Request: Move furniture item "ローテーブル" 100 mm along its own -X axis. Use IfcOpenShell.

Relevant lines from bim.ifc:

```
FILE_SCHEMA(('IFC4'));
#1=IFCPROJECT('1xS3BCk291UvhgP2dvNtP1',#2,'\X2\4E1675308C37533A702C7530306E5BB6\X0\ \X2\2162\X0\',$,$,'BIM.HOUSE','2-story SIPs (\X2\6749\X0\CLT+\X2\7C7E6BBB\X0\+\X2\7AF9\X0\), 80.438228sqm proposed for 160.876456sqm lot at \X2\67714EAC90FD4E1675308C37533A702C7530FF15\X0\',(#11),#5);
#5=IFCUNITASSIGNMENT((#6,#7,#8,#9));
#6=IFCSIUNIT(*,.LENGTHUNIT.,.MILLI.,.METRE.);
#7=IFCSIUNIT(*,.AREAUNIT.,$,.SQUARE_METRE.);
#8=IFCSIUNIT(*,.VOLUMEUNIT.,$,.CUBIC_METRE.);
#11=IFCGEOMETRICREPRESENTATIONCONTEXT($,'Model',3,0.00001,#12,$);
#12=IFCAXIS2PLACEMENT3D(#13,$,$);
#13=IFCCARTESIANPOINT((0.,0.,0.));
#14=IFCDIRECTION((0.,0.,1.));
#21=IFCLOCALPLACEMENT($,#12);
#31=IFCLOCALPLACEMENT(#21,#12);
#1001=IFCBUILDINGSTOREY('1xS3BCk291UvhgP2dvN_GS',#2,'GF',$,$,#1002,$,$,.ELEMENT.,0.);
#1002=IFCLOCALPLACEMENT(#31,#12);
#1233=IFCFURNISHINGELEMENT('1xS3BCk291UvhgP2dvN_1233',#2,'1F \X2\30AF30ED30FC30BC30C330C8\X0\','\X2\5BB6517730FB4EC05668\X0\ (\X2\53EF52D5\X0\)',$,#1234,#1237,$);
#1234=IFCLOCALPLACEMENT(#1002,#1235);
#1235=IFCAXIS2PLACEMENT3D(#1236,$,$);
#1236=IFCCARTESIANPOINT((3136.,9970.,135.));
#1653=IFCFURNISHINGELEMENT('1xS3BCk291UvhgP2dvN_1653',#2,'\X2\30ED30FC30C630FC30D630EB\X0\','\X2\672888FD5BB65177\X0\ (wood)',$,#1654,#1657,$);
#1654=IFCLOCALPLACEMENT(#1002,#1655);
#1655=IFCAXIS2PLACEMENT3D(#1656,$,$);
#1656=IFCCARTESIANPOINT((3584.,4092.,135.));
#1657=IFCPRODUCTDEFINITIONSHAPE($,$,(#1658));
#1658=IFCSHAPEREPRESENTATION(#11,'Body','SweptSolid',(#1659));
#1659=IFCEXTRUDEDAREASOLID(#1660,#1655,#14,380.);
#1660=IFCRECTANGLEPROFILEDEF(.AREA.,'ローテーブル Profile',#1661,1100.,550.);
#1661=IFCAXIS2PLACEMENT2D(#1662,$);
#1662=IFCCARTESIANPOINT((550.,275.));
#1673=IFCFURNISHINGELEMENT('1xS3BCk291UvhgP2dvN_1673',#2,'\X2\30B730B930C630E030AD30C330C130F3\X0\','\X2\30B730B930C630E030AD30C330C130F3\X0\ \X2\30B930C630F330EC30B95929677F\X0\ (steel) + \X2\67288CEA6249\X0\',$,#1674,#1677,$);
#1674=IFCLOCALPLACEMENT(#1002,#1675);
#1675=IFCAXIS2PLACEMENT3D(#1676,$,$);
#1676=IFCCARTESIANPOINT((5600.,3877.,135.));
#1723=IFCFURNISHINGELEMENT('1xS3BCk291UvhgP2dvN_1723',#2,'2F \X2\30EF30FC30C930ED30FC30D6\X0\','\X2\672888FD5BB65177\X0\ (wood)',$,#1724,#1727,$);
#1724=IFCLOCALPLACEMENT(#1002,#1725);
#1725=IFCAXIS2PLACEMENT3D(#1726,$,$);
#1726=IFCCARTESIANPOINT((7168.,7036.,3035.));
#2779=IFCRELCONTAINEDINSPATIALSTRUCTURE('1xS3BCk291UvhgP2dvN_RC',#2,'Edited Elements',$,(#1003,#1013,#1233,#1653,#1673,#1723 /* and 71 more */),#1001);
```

```python
import ifcopenshell
import ifcopenshell.api.geometry
import ifcopenshell.util.placement

model = ifcopenshell.open("bim.ifc")

item = model.by_guid("1xS3BCk291UvhgP2dvN_1653")
matrix = ifcopenshell.util.placement.get_local_placement(item.ObjectPlacement)
matrix[:3, 3] -= matrix[:3, 0] * 100.0
ifcopenshell.api.geometry.edit_object_placement(model, product=item, matrix=matrix, is_si=False)

print(ifcopenshell.util.placement.get_local_placement(item.ObjectPlacement).round(3) + 0.0)

model.write("bim_v2.ifc")
```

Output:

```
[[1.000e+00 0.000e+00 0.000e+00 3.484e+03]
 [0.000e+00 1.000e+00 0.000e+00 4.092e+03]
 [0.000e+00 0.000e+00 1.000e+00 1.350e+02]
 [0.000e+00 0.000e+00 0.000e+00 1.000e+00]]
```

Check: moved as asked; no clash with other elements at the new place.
